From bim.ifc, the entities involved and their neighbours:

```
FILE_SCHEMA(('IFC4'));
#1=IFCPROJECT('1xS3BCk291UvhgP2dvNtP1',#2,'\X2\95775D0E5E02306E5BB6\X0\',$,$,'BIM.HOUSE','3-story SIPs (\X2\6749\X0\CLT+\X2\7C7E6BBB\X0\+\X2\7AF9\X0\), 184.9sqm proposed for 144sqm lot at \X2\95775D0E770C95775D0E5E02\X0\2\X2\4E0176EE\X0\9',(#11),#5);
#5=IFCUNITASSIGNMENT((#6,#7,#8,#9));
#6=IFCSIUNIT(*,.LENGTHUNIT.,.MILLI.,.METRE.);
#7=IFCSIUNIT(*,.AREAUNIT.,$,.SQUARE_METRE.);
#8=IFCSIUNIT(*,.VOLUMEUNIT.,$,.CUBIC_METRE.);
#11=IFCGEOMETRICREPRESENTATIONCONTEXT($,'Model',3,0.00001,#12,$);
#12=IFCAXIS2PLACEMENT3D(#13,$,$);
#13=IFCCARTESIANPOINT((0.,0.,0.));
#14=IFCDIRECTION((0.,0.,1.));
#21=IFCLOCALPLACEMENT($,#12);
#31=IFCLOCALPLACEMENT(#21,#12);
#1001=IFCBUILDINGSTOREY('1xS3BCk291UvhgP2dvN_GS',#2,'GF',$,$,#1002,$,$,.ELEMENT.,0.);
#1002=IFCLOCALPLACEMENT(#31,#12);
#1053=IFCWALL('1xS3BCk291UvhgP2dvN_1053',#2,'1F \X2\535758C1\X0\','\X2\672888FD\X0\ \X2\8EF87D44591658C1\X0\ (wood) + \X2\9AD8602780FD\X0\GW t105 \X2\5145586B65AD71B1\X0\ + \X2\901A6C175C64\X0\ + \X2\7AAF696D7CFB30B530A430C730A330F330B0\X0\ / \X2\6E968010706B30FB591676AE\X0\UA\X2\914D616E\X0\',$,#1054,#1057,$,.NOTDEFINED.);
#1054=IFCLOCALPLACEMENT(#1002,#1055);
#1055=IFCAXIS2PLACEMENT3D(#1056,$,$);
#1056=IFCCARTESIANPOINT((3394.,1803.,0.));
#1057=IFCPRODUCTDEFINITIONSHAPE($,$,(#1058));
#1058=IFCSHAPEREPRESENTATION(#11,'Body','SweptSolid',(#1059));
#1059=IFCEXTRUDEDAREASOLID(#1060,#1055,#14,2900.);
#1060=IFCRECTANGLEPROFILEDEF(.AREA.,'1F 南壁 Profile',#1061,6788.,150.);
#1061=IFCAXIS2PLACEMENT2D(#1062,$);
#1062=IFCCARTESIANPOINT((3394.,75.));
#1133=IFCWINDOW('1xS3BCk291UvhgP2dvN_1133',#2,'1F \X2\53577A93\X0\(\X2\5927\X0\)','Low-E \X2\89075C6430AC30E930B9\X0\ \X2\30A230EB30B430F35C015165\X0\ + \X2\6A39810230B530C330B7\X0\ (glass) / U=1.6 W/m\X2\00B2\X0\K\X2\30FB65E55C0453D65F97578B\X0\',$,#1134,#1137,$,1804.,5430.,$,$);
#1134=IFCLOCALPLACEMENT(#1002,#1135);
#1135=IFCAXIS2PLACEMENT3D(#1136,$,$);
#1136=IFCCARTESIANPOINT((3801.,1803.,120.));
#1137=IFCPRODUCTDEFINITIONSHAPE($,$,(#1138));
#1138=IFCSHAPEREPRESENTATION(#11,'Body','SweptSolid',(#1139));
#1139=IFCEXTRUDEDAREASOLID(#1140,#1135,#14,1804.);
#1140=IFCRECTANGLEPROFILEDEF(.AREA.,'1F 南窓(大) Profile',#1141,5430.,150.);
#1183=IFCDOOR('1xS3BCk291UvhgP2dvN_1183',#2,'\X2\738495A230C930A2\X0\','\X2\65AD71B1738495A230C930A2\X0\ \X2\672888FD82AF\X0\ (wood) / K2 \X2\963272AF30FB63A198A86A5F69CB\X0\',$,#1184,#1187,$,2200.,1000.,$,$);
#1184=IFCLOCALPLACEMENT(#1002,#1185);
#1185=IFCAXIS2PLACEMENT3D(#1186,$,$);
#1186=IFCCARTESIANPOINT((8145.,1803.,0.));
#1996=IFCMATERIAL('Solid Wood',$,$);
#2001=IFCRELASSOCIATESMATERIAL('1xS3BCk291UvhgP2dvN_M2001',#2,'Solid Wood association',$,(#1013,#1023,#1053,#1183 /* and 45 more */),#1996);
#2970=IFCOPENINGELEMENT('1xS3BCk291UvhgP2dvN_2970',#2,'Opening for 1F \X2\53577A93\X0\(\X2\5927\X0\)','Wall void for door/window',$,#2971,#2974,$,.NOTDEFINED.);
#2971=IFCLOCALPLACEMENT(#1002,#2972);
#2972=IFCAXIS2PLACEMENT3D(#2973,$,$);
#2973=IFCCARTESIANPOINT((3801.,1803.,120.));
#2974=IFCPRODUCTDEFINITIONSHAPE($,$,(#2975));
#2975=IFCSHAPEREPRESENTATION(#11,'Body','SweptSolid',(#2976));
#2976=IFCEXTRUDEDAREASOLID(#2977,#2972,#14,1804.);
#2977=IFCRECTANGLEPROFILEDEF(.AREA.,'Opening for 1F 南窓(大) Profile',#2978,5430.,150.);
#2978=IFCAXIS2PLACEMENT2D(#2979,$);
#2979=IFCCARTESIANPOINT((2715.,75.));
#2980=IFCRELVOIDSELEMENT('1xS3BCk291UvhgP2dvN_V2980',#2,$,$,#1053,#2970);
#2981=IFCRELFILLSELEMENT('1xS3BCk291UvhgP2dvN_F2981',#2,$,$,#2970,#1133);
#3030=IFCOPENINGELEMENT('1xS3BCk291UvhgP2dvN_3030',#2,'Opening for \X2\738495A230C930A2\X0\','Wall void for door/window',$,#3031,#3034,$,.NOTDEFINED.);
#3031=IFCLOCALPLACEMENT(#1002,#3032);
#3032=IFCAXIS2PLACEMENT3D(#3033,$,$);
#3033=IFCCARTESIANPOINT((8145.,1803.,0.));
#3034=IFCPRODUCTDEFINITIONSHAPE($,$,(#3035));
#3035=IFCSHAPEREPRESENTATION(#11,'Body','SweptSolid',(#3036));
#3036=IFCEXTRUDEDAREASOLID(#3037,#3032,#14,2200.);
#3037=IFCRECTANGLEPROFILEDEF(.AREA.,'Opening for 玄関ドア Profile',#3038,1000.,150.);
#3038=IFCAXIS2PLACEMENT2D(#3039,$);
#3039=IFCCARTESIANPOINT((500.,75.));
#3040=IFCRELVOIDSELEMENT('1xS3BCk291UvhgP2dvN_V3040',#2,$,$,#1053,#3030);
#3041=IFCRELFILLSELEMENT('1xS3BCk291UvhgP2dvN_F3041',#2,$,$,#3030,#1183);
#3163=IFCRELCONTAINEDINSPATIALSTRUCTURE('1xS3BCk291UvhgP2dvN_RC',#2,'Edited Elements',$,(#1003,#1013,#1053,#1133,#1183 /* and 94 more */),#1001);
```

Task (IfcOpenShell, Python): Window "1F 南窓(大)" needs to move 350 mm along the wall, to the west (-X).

```python
import ifcopenshell
import ifcopenshell.api.geometry
import ifcopenshell.util.placement
import ifcopenshell.util.unit

model = ifcopenshell.open("bim.ifc")
unit_scale = ifcopenshell.util.unit.calculate_unit_scale(model)

window = model.by_guid("1xS3BCk291UvhgP2dvN_1133")
opening = window.FillsVoids[0].RelatingOpeningElement
wall = opening.VoidsElements[0].RelatingBuildingElement

wall_matrix = ifcopenshell.util.placement.get_local_placement(wall.ObjectPlacement)
shift = wall_matrix[:3, 0] * -0.35 / unit_scale
before = ifcopenshell.util.placement.get_local_placement(window.ObjectPlacement)[:3, 3].copy()

# The window is not placed relative to its opening, so move both.
for product in (opening, window):
    matrix = ifcopenshell.util.placement.get_local_placement(product.ObjectPlacement)
    matrix[:3, 3] += shift
    ifcopenshell.api.geometry.edit_object_placement(model, product=product, matrix=matrix, is_si=False)

after = ifcopenshell.util.placement.get_local_placement(window.ObjectPlacement)[:3, 3]
print("window moved by", (after - before).round(3) + 0.0)

model.write("bim_rev.ifc")
```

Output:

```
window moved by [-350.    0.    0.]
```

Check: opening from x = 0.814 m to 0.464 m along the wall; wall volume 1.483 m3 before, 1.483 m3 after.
